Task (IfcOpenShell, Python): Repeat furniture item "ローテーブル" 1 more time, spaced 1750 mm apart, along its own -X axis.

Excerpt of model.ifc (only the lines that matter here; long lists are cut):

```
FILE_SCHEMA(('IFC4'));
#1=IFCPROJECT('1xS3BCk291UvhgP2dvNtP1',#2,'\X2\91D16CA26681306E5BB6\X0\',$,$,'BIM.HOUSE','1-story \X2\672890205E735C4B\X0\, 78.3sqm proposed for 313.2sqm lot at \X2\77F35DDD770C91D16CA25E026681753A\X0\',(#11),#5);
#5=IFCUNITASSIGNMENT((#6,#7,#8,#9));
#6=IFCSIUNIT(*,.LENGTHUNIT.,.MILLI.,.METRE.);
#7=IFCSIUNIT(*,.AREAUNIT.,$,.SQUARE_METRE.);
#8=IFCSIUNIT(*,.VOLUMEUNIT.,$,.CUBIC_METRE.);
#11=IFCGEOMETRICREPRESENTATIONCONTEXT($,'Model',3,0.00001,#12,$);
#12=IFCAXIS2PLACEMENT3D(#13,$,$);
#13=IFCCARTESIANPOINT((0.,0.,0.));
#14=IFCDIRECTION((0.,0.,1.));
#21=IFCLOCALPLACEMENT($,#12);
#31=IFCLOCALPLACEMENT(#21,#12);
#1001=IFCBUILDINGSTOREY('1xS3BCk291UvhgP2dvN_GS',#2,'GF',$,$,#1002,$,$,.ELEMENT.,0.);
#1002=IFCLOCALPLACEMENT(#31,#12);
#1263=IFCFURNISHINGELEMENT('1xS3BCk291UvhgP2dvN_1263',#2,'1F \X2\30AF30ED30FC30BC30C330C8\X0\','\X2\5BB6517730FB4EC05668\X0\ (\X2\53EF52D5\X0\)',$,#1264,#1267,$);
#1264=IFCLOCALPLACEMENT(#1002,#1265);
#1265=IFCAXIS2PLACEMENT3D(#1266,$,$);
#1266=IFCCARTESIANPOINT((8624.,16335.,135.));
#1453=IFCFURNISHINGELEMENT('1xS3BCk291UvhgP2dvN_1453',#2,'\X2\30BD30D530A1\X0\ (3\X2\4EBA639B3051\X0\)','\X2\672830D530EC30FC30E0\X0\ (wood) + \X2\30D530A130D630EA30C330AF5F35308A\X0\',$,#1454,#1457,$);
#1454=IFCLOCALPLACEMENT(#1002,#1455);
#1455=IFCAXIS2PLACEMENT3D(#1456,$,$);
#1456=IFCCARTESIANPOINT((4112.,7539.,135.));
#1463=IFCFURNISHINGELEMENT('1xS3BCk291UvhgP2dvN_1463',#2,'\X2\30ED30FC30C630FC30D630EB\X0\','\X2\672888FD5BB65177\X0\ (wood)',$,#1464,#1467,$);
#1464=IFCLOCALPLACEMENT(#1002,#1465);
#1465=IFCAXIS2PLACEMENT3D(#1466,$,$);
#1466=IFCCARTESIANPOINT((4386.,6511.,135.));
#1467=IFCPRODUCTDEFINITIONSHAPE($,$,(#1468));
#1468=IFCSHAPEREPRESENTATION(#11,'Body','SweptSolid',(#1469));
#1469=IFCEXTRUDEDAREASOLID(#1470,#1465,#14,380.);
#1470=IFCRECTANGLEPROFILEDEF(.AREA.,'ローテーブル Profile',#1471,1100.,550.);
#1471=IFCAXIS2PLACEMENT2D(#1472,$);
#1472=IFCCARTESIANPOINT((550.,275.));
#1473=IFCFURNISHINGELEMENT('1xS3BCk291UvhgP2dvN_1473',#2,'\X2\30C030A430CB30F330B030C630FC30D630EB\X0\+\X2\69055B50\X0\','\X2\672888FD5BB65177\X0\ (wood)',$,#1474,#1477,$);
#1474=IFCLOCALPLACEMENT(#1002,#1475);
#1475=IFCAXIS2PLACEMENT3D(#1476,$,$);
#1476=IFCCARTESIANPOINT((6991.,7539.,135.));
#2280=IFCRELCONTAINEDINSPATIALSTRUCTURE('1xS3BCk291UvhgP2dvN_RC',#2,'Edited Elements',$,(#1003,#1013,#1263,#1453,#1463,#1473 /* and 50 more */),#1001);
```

```python
import ifcopenshell
import ifcopenshell.api.geometry
import ifcopenshell.api.root
import ifcopenshell.util.element
import ifcopenshell.util.placement

model = ifcopenshell.open("model.ifc")


def reuse_history(source, copy):
    """copy_class also copies each property set's owner history, people and application; keep the originals."""
    for rel in copy.IsDefinedBy:
        if rel.is_a("IfcRelDefinesByProperties") and (history := rel.RelatingPropertyDefinition.OwnerHistory):
            rel.RelatingPropertyDefinition.OwnerHistory = source.OwnerHistory
            ifcopenshell.util.element.remove_deep2(model, history)


source = model.by_guid("1xS3BCk291UvhgP2dvN_1463")
base = ifcopenshell.util.placement.get_local_placement(source.ObjectPlacement)
step = -base[:3, 0] * 1750.0

for i in range(1, 2):
    copy = ifcopenshell.api.root.copy_class(model, product=source)
    copy.Representation = ifcopenshell.util.element.copy_deep(
        model, source.Representation, exclude=["IfcGeometricRepresentationContext", "IfcRepresentationMap"]
    )
    reuse_history(source, copy)
    matrix = base.copy()
    matrix[:3, 3] += i * step
    print("added at", matrix[:3, 3].round(3) + 0.0)
    ifcopenshell.api.geometry.edit_object_placement(model, product=copy, matrix=matrix, is_si=False)

model.write("model_rev.ifc")
```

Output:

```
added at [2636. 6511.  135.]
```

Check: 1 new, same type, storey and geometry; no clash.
